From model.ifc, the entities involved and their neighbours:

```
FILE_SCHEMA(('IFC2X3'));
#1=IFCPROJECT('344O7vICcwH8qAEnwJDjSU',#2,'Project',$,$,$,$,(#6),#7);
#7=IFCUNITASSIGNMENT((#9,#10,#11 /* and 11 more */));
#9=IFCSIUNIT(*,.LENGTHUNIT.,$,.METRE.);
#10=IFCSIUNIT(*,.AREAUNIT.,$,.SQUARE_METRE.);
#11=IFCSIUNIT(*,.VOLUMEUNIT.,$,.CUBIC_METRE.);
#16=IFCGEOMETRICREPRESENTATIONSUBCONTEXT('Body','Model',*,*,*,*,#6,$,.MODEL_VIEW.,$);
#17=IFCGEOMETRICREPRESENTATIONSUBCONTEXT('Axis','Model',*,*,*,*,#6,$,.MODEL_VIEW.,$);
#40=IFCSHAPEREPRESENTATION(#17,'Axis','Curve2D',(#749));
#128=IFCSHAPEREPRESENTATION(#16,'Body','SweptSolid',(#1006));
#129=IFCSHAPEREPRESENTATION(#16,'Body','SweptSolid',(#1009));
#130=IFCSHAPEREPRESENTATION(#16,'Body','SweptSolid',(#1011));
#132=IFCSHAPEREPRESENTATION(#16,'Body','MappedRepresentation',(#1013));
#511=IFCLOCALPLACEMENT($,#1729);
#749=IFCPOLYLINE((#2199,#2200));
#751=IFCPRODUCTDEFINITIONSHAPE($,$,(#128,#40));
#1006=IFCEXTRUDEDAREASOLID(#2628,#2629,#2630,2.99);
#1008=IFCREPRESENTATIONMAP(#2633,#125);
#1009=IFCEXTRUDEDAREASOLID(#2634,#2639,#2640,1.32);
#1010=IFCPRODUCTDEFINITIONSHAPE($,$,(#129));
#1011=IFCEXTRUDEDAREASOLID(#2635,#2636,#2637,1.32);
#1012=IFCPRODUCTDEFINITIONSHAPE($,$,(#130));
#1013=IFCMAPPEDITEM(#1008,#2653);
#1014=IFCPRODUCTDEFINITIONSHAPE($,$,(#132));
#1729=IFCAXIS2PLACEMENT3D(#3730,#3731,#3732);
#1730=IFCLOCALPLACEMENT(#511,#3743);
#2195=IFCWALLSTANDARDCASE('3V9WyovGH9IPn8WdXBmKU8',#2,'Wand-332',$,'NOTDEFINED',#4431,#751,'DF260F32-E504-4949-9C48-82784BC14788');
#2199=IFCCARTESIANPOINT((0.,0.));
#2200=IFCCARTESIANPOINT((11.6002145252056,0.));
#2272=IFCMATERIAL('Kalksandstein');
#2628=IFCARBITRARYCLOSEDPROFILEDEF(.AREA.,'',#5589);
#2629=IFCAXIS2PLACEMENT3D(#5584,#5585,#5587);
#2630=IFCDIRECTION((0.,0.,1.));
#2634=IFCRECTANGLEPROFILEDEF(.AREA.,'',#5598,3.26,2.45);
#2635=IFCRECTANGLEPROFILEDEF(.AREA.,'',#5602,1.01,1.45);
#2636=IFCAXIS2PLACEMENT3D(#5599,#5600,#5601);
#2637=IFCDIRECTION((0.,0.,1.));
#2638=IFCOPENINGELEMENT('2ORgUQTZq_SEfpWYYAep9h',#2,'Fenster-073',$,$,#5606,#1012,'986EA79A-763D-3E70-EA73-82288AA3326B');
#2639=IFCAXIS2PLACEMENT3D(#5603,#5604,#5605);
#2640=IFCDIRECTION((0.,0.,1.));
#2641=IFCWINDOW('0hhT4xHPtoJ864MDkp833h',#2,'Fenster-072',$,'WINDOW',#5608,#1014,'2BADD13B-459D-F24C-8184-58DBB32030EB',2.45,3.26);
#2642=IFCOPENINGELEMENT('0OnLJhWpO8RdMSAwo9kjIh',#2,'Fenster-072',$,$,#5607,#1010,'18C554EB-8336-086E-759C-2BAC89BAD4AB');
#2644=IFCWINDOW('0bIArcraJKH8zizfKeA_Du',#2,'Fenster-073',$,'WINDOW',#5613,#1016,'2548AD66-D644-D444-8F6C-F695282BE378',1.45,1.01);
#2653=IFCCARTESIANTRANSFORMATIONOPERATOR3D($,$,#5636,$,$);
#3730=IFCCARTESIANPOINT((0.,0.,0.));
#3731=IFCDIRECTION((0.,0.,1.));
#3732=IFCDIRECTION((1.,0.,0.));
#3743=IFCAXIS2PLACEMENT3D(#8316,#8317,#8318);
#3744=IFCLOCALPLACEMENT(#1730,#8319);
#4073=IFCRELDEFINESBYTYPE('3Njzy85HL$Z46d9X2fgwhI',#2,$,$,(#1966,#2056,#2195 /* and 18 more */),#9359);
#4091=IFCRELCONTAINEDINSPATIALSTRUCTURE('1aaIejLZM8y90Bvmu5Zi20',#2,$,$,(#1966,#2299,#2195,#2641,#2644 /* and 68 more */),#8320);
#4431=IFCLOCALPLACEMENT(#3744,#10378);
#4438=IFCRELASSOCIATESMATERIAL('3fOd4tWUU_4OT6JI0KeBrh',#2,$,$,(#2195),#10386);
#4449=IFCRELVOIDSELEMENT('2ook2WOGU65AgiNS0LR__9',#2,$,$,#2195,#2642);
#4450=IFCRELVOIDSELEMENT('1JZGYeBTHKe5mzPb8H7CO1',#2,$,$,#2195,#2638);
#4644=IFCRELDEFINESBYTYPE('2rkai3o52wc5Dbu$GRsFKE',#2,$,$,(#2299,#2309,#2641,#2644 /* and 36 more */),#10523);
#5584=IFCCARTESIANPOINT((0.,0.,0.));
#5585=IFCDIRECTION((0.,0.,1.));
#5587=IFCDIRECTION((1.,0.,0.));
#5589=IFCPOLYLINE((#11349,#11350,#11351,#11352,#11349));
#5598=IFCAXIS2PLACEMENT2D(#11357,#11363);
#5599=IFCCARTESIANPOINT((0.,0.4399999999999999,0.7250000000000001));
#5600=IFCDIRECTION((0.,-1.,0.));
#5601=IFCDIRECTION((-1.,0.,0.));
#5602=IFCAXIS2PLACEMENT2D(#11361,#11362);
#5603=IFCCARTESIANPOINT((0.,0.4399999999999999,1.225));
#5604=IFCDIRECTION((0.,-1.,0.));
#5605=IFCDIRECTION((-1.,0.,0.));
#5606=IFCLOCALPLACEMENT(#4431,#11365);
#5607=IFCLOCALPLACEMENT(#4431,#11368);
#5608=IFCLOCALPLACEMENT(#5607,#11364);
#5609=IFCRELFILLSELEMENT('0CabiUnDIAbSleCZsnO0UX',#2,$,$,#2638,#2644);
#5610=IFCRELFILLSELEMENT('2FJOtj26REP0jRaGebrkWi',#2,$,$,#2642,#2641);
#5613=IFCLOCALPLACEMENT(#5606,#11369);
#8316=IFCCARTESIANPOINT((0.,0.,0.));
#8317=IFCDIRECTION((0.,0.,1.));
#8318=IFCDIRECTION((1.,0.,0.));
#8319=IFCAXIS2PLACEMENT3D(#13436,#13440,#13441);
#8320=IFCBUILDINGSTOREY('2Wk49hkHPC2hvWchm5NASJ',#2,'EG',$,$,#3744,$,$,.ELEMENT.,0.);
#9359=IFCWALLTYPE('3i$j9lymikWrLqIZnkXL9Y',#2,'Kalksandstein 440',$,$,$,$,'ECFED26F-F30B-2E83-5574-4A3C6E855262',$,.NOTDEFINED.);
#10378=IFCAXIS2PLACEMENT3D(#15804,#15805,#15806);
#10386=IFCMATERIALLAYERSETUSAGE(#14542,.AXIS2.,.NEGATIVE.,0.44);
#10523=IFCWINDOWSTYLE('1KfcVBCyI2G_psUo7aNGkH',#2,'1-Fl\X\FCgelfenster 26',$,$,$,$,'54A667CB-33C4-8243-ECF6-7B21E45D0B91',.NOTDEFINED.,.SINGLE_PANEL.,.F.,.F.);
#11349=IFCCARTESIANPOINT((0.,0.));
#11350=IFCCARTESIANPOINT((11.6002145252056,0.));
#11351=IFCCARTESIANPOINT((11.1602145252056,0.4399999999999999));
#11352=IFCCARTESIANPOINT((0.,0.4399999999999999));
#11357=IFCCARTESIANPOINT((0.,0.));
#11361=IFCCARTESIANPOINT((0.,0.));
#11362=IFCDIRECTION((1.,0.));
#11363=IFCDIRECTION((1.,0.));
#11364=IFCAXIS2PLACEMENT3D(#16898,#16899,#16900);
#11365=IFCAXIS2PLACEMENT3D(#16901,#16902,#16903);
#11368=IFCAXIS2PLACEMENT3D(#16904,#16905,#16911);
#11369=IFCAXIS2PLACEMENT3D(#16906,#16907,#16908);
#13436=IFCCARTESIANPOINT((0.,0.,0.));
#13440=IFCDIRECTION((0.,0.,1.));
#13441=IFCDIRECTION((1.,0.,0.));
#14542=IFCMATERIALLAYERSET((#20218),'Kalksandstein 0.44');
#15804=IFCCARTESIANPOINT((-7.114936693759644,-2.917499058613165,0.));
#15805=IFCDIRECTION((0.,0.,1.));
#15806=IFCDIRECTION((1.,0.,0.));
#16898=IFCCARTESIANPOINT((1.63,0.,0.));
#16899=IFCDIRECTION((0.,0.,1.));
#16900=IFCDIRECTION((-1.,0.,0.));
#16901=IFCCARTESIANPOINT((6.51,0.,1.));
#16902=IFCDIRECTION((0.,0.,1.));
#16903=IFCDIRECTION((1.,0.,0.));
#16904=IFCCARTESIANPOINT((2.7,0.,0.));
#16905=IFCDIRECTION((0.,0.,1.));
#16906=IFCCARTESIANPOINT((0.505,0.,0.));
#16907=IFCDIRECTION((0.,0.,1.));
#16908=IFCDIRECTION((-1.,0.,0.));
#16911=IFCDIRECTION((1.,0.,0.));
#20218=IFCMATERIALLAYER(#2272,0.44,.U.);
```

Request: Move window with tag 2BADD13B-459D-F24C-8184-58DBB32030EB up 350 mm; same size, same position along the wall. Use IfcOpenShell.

```python
import numpy as np
import ifcopenshell
import ifcopenshell.api.geometry
import ifcopenshell.util.placement
import ifcopenshell.util.unit

model = ifcopenshell.open("model.ifc")
unit_scale = ifcopenshell.util.unit.calculate_unit_scale(model)

window = model.by_guid("0hhT4xHPtoJ864MDkp833h")
opening = window.FillsVoids[0].RelatingOpeningElement
dz = 0.35 / unit_scale

shift = np.array([0.0, 0.0, dz])
# The window is placed relative to its opening, so it follows when the opening moves.
matrix = ifcopenshell.util.placement.get_local_placement(opening.ObjectPlacement)
matrix[:3, 3] += shift
ifcopenshell.api.geometry.edit_object_placement(
    model, product=opening, matrix=matrix, is_si=False, should_transform_children=True
)

print(f"moved by {dz * unit_scale:+.3f} m")

model.write("model-out.ifc")
```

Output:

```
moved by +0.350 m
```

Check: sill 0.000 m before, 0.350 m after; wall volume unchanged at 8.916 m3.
